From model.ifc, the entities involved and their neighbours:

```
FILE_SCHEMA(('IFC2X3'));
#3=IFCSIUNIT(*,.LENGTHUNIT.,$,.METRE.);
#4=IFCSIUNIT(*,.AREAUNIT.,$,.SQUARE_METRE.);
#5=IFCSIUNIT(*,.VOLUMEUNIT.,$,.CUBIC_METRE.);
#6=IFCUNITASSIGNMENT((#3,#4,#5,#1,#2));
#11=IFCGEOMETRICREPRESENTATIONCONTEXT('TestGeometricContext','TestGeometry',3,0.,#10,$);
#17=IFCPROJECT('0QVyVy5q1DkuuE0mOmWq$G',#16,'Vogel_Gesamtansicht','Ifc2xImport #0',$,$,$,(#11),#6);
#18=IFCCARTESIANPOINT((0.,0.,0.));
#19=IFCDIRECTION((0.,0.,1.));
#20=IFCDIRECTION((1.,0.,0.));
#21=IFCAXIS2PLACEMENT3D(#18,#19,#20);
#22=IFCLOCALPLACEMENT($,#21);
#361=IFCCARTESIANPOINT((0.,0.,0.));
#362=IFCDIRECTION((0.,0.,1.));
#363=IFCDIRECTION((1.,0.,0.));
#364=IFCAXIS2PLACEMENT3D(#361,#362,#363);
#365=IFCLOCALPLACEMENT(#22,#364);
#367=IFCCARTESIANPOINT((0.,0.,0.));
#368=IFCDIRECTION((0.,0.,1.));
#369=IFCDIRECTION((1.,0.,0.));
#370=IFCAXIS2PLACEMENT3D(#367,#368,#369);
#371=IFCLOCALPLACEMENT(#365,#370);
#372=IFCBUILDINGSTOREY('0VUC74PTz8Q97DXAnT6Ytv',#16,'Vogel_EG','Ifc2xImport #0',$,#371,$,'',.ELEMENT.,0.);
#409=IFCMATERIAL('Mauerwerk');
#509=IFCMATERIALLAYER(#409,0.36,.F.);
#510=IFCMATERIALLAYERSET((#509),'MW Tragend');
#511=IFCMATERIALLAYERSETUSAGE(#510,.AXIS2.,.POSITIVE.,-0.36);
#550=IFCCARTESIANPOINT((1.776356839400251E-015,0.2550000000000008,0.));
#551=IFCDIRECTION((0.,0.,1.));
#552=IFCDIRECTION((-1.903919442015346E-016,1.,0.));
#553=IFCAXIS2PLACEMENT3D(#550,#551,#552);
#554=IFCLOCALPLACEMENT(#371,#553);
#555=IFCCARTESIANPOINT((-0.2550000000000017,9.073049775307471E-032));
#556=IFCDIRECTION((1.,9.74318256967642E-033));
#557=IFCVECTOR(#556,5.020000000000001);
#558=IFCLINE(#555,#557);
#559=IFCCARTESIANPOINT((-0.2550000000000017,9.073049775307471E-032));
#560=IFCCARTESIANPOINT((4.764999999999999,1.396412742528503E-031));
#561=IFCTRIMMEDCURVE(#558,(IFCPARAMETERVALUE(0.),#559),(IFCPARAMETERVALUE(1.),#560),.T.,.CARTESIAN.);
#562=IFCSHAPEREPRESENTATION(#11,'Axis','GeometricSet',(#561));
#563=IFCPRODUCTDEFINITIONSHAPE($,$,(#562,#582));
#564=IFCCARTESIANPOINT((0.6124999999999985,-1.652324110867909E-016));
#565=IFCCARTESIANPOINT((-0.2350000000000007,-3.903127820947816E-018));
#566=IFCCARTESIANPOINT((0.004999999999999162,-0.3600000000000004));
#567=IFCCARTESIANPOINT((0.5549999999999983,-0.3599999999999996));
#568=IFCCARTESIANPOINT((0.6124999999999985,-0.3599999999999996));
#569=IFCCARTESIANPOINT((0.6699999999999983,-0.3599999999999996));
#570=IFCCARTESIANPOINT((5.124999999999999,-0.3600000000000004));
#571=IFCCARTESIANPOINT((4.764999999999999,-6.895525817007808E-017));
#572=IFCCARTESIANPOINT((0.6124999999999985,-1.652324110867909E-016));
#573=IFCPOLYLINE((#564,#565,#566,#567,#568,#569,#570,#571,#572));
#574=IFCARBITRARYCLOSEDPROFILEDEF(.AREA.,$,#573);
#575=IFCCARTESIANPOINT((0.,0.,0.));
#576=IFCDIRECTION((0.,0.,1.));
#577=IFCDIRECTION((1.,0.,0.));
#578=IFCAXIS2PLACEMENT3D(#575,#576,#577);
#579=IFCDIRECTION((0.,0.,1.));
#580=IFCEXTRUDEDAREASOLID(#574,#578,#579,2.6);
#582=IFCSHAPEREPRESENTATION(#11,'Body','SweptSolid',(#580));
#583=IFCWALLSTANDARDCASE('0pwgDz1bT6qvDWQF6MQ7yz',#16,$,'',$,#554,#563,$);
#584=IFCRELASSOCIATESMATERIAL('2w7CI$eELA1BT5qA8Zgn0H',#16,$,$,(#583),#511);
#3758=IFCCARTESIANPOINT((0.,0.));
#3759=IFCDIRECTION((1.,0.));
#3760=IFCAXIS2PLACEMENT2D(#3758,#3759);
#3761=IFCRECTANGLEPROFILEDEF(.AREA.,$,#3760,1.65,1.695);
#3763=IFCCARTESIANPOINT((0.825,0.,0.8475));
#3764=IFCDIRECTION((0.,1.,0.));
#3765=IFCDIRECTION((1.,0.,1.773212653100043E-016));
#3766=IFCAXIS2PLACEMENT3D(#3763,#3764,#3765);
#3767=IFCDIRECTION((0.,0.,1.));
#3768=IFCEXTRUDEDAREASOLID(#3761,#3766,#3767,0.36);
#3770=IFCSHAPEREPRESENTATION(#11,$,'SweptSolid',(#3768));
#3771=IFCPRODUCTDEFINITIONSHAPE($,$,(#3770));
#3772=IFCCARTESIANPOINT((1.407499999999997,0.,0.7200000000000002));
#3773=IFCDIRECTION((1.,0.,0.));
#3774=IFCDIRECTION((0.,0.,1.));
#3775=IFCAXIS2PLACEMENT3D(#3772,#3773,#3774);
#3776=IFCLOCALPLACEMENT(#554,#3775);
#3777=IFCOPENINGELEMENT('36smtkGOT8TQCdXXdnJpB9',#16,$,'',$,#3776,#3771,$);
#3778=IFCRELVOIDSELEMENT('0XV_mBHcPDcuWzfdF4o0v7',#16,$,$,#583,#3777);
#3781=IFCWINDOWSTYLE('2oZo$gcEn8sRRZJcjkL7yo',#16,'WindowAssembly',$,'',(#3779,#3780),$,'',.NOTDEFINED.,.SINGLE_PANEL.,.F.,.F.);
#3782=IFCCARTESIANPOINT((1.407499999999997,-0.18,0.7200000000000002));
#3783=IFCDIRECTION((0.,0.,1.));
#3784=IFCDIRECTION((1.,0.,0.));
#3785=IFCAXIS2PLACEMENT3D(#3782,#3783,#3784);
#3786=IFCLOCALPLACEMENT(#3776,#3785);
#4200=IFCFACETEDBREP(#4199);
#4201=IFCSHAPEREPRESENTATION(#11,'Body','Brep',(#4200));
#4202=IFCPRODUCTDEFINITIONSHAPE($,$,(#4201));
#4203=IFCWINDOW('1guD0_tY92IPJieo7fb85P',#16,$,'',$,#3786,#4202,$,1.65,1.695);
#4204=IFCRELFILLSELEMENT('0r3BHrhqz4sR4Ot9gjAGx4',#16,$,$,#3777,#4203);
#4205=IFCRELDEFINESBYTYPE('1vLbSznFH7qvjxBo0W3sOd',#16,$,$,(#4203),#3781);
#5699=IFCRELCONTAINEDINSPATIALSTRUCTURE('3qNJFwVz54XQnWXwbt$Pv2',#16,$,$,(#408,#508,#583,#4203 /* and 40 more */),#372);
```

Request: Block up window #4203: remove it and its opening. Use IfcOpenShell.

```python
import ifcopenshell
import ifcopenshell.api.feature
import ifcopenshell.api.root
import ifcopenshell.geom
import ifcopenshell.util.shape

model = ifcopenshell.open("model.ifc")
settings = ifcopenshell.geom.settings()


def volume(element):
    """Net volume in cubic metres, openings subtracted."""
    shape = ifcopenshell.geom.create_shape(settings, element)
    return ifcopenshell.util.shape.get_volume(shape.geometry)


window = model.by_id(4203)
opening = window.FillsVoids[0].RelatingOpeningElement
wall = opening.VoidsElements[0].RelatingBuildingElement
before = volume(wall)

ifcopenshell.api.root.remove_product(model, product=window)
ifcopenshell.api.feature.remove_feature(model, feature=opening)

after = volume(wall)

print(f"wall volume {before:.3f} -> {after:.3f} m3")

model.write("model_edited.ifc")
```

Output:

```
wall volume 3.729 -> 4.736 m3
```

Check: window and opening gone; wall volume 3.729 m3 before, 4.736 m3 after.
